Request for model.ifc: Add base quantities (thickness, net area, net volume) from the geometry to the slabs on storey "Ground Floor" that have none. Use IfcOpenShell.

First a look at what the model holds.

```python
import ifcopenshell
import ifcopenshell.util.element
import ifcopenshell.util.unit

model = ifcopenshell.open("model.ifc")
print(model.schema)
for unit_type in ("LENGTHUNIT", "AREAUNIT", "VOLUMEUNIT"):
    print(unit_type, ifcopenshell.util.unit.calculate_unit_scale(model, unit_type))
storey = next(s for s in model.by_type("IfcBuildingStorey") if s.Name == "Ground Floor")
slabs = [e for e in ifcopenshell.util.element.get_decomposition(storey) if e.is_a("IfcSlab")]
for e in sorted(slabs, key=lambda e: e.id()):
    print(e.id(), e.is_a(), e.Name, list(ifcopenshell.util.element.get_psets(e, qtos_only=True)), sep=" | ")
```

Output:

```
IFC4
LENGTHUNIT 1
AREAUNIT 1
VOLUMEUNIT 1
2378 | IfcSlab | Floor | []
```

```python
import ifcopenshell
import ifcopenshell.api.pset
import ifcopenshell.geom
import ifcopenshell.util.element
import ifcopenshell.util.shape
import ifcopenshell.util.unit

model = ifcopenshell.open("model.ifc")
unit_scale = ifcopenshell.util.unit.calculate_unit_scale(model)
area_scale = ifcopenshell.util.unit.calculate_unit_scale(model, "AREAUNIT")
volume_scale = ifcopenshell.util.unit.calculate_unit_scale(model, "VOLUMEUNIT")
settings = ifcopenshell.geom.settings()

storey = next(s for s in model.by_type("IfcBuildingStorey") if s.Name == "Ground Floor")
slabs = [e for e in ifcopenshell.util.element.get_decomposition(storey) if e.is_a("IfcSlab")]

for e in sorted(slabs, key=lambda e: e.id()):
    if ifcopenshell.util.element.get_psets(e, qtos_only=True, should_inherit=False):
        continue
    # Geometry comes back in metres, in the element's own axes.
    shape = ifcopenshell.geom.create_shape(settings, e)
    values = {
        "Width": ifcopenshell.util.shape.get_z(shape.geometry) / unit_scale,
        "NetArea": ifcopenshell.util.shape.get_footprint_area(shape.geometry) / area_scale,
        "NetVolume": ifcopenshell.util.shape.get_volume(shape.geometry) / volume_scale,
    }
    qto = ifcopenshell.api.pset.add_qto(model, product=e, name="Qto_SlabBaseQuantities")
    ifcopenshell.api.pset.edit_qto(model, qto=qto, properties=values)
    print(e.id(), {k: round(v, 3) for k, v in values.items()})

model.write("model_v2.ifc")
```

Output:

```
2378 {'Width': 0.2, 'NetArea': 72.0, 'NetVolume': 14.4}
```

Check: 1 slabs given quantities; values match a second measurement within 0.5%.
